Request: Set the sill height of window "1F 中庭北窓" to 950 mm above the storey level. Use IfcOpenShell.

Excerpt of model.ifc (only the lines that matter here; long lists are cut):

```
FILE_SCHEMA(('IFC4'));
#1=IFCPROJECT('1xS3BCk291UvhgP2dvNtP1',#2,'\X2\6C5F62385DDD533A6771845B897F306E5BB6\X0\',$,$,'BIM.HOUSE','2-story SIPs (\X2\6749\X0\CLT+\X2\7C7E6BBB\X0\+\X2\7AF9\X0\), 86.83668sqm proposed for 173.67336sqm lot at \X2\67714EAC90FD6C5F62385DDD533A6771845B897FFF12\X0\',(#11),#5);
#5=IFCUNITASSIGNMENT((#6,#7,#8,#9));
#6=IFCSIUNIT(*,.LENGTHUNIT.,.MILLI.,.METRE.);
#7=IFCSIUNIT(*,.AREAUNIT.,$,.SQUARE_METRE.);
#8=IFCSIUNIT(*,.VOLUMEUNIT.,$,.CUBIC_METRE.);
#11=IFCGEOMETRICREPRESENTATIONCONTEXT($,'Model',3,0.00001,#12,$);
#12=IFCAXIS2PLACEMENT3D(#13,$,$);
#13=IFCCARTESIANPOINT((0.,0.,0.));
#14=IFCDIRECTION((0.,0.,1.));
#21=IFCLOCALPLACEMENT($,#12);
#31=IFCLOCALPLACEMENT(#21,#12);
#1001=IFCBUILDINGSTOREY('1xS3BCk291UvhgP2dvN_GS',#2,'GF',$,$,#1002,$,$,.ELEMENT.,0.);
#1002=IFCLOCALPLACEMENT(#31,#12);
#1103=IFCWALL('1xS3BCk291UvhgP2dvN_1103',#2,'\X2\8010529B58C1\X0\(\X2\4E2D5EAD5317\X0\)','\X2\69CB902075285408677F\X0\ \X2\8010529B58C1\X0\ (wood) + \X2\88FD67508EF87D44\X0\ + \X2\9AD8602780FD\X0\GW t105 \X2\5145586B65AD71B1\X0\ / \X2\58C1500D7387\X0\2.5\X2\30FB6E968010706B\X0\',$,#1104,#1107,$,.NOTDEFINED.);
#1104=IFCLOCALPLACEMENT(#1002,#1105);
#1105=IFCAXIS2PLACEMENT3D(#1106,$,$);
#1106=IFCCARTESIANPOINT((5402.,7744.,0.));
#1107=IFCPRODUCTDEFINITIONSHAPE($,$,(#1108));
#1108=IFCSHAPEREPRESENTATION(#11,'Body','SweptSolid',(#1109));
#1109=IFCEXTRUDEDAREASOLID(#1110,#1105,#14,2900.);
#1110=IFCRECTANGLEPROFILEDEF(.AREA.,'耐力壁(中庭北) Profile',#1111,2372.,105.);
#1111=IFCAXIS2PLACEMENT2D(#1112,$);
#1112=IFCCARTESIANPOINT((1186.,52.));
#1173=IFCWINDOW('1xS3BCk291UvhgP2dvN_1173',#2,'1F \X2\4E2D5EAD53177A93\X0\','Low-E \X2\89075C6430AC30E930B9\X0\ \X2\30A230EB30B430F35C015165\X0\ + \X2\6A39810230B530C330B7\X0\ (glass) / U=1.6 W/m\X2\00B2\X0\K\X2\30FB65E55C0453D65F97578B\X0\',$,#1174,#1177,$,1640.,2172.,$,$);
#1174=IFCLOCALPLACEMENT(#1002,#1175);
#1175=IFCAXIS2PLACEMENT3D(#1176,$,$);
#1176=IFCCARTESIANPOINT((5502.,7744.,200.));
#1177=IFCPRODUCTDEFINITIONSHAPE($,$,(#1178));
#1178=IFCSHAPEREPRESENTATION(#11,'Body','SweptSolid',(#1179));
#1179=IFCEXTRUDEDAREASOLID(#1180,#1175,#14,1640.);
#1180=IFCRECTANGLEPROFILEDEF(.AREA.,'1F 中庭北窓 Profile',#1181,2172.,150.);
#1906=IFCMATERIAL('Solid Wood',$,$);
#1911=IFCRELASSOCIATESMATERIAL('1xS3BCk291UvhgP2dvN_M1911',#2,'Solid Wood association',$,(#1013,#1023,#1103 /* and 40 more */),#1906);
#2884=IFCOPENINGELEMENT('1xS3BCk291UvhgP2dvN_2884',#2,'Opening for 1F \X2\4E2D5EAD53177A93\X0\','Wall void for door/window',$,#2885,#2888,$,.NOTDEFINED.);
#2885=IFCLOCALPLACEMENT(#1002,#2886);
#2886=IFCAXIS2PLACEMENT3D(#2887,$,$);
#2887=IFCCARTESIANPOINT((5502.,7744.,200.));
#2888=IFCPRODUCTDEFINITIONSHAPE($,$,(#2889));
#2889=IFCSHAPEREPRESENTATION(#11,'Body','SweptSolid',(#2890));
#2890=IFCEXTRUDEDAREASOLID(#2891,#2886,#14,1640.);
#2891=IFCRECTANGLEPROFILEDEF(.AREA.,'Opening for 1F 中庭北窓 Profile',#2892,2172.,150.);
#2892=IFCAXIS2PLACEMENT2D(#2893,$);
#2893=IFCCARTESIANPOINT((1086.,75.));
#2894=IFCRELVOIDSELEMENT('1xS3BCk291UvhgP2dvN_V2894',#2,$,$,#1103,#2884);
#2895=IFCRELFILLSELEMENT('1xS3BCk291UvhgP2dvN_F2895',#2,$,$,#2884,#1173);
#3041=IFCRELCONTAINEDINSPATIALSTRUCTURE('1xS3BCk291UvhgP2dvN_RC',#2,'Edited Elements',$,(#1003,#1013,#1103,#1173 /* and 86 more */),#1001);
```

```python
import numpy as np
import ifcopenshell
import ifcopenshell.api.geometry
import ifcopenshell.geom
import ifcopenshell.util.element
import ifcopenshell.util.placement
import ifcopenshell.util.shape
import ifcopenshell.util.unit

model = ifcopenshell.open("model.ifc")
unit_scale = ifcopenshell.util.unit.calculate_unit_scale(model)

window = model.by_guid("1xS3BCk291UvhgP2dvN_1173")
opening = window.FillsVoids[0].RelatingOpeningElement
storey = ifcopenshell.util.element.get_container(window, ifc_class="IfcBuildingStorey")
level = ifcopenshell.util.placement.get_local_placement(storey.ObjectPlacement)[2, 3]

# The opening's origin need not be at the sill, so measure its lowest point.
shape = ifcopenshell.geom.create_shape(ifcopenshell.geom.settings(), opening)
bottom = ifcopenshell.util.shape.get_shape_bottom_elevation(shape, shape.geometry) / unit_scale
dz = level + 0.95 / unit_scale - bottom

shift = np.array([0.0, 0.0, dz])
# The window is not placed relative to its opening, so move both.
for product in (opening, window):
    matrix = ifcopenshell.util.placement.get_local_placement(product.ObjectPlacement)
    matrix[:3, 3] += shift
    ifcopenshell.api.geometry.edit_object_placement(model, product=product, matrix=matrix, is_si=False)

print(f"moved by {dz * unit_scale:+.3f} m")

model.write("model_v2.ifc")
```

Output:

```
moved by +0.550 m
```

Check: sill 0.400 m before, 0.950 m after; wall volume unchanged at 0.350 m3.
